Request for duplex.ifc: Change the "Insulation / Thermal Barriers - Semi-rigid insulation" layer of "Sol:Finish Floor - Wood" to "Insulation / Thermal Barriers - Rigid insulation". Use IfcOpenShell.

First a look at what the model holds.

```python
import ifcopenshell
import ifcopenshell.util.element

model = ifcopenshell.open("duplex.ifc")
print(model.schema)
for layer_set in model.by_type("IfcMaterialLayerSet"):
    if layer_set.LayerSetName == "Sol:Finish Floor - Wood":
        for layer in layer_set.MaterialLayers:
            print(layer.id(), layer.Material and layer.Material.Name, layer.LayerThickness, sep=" | ")
        print(len(ifcopenshell.util.element.get_elements_by_material(model, layer_set)), "elements and types use it")
print(sorted(m.Name for m in model.by_type("IfcMaterial") if m.Name)[:60])
```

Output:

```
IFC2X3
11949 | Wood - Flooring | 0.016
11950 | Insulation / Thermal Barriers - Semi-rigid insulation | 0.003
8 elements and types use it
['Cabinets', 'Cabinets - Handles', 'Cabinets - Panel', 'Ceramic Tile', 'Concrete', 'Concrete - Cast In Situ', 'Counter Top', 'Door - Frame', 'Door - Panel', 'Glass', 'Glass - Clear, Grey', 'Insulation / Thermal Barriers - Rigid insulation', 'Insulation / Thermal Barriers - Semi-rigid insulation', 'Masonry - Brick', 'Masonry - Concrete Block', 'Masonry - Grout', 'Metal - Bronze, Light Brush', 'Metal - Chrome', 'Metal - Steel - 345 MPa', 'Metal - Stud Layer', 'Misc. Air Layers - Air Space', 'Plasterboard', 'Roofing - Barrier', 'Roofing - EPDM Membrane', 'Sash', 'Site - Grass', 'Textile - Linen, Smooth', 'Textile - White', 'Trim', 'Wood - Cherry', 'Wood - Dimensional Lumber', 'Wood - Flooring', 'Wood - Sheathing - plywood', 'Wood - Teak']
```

```python
import ifcopenshell
import ifcopenshell.api.material

model = ifcopenshell.open("duplex.ifc")

layer_set = next(s for s in model.by_type("IfcMaterialLayerSet") if s.LayerSetName == "Sol:Finish Floor - Wood")
layer = next(l for l in layer_set.MaterialLayers if l.Material and l.Material.Name == "Insulation / Thermal Barriers - Semi-rigid insulation")
material = next(m for m in model.by_type("IfcMaterial") if m.Name == "Insulation / Thermal Barriers - Rigid insulation")

# Point this one layer at the other material; renaming the old one would change it everywhere.
ifcopenshell.api.material.edit_layer(model, layer=layer, attributes={}, material=material)

print([l.Material.Name if l.Material else None for l in layer_set.MaterialLayers])

model.write("duplex_updated.ifc")
```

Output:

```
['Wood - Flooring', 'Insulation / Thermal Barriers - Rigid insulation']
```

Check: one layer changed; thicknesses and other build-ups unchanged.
